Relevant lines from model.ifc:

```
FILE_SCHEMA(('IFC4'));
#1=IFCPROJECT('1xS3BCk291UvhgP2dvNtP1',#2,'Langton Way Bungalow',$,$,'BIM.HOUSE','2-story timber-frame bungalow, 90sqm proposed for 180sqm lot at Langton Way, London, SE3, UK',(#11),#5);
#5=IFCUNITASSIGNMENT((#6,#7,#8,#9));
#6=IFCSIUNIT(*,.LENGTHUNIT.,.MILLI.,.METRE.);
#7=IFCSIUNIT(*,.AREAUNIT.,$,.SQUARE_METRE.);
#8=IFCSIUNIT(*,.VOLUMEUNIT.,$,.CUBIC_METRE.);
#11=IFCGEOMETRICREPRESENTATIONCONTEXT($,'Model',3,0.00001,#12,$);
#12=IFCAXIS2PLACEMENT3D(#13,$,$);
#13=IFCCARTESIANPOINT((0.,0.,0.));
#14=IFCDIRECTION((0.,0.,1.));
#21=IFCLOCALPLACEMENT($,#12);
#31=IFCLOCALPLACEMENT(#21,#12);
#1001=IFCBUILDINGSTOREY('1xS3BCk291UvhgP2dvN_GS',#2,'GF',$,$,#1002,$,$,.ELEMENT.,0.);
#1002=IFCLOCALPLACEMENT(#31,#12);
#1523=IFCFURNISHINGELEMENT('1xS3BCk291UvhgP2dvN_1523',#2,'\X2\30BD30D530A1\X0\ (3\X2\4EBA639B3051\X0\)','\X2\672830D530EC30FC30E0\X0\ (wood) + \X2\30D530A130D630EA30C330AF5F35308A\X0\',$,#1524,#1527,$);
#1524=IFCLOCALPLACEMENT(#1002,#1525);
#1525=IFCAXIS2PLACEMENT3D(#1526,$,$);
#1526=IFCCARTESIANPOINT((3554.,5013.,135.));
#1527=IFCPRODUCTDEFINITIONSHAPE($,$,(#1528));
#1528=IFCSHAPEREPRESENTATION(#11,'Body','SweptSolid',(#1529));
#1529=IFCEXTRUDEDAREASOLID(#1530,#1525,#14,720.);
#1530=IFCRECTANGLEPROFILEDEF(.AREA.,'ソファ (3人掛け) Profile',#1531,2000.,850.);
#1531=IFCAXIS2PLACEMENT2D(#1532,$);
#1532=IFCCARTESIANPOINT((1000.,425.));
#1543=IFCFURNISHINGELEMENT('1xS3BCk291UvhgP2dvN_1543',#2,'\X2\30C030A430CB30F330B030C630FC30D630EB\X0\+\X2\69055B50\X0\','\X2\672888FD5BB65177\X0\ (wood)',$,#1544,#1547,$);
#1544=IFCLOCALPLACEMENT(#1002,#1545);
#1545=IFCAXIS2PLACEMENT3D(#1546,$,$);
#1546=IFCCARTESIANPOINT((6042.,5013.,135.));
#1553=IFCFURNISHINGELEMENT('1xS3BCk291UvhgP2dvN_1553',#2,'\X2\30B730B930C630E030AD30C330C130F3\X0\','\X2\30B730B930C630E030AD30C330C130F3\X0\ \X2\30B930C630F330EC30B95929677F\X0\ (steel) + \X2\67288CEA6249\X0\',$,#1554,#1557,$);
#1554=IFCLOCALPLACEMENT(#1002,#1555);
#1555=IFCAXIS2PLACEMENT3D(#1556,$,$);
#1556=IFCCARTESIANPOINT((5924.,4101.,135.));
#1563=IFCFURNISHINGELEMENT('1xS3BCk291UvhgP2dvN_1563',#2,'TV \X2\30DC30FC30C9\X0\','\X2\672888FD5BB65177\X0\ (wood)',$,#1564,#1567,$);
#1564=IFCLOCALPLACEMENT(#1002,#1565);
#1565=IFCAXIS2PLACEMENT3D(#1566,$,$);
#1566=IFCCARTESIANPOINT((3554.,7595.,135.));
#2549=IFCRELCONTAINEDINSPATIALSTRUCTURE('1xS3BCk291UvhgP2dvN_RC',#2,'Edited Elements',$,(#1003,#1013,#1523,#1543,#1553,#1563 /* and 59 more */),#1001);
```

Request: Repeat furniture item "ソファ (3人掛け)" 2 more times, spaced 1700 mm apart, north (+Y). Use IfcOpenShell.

```python
import numpy as np
import ifcopenshell
import ifcopenshell.api.geometry
import ifcopenshell.api.root
import ifcopenshell.util.element
import ifcopenshell.util.placement
import ifcopenshell.util.unit

model = ifcopenshell.open("model.ifc")
unit_scale = ifcopenshell.util.unit.calculate_unit_scale(model)


def reuse_history(source, copy):
    """copy_class also copies each property set's owner history, people and application; keep the originals."""
    for rel in copy.IsDefinedBy:
        if rel.is_a("IfcRelDefinesByProperties") and (history := rel.RelatingPropertyDefinition.OwnerHistory):
            rel.RelatingPropertyDefinition.OwnerHistory = source.OwnerHistory
            ifcopenshell.util.element.remove_deep2(model, history)


source = model.by_guid("1xS3BCk291UvhgP2dvN_1523")
base = ifcopenshell.util.placement.get_local_placement(source.ObjectPlacement)
step = np.array([0.0, 1.0, 0.0]) * 1.7 / unit_scale

for i in range(1, 3):
    copy = ifcopenshell.api.root.copy_class(model, product=source)
    copy.Representation = ifcopenshell.util.element.copy_deep(
        model, source.Representation, exclude=["IfcGeometricRepresentationContext", "IfcRepresentationMap"]
    )
    reuse_history(source, copy)
    matrix = base.copy()
    matrix[:3, 3] += i * step
    print("added at", matrix[:3, 3].round(3) + 0.0)
    ifcopenshell.api.geometry.edit_object_placement(model, product=copy, matrix=matrix, is_si=False)

model.write("model_edited.ifc")
```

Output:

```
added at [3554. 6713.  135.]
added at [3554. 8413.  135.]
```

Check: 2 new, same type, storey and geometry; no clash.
